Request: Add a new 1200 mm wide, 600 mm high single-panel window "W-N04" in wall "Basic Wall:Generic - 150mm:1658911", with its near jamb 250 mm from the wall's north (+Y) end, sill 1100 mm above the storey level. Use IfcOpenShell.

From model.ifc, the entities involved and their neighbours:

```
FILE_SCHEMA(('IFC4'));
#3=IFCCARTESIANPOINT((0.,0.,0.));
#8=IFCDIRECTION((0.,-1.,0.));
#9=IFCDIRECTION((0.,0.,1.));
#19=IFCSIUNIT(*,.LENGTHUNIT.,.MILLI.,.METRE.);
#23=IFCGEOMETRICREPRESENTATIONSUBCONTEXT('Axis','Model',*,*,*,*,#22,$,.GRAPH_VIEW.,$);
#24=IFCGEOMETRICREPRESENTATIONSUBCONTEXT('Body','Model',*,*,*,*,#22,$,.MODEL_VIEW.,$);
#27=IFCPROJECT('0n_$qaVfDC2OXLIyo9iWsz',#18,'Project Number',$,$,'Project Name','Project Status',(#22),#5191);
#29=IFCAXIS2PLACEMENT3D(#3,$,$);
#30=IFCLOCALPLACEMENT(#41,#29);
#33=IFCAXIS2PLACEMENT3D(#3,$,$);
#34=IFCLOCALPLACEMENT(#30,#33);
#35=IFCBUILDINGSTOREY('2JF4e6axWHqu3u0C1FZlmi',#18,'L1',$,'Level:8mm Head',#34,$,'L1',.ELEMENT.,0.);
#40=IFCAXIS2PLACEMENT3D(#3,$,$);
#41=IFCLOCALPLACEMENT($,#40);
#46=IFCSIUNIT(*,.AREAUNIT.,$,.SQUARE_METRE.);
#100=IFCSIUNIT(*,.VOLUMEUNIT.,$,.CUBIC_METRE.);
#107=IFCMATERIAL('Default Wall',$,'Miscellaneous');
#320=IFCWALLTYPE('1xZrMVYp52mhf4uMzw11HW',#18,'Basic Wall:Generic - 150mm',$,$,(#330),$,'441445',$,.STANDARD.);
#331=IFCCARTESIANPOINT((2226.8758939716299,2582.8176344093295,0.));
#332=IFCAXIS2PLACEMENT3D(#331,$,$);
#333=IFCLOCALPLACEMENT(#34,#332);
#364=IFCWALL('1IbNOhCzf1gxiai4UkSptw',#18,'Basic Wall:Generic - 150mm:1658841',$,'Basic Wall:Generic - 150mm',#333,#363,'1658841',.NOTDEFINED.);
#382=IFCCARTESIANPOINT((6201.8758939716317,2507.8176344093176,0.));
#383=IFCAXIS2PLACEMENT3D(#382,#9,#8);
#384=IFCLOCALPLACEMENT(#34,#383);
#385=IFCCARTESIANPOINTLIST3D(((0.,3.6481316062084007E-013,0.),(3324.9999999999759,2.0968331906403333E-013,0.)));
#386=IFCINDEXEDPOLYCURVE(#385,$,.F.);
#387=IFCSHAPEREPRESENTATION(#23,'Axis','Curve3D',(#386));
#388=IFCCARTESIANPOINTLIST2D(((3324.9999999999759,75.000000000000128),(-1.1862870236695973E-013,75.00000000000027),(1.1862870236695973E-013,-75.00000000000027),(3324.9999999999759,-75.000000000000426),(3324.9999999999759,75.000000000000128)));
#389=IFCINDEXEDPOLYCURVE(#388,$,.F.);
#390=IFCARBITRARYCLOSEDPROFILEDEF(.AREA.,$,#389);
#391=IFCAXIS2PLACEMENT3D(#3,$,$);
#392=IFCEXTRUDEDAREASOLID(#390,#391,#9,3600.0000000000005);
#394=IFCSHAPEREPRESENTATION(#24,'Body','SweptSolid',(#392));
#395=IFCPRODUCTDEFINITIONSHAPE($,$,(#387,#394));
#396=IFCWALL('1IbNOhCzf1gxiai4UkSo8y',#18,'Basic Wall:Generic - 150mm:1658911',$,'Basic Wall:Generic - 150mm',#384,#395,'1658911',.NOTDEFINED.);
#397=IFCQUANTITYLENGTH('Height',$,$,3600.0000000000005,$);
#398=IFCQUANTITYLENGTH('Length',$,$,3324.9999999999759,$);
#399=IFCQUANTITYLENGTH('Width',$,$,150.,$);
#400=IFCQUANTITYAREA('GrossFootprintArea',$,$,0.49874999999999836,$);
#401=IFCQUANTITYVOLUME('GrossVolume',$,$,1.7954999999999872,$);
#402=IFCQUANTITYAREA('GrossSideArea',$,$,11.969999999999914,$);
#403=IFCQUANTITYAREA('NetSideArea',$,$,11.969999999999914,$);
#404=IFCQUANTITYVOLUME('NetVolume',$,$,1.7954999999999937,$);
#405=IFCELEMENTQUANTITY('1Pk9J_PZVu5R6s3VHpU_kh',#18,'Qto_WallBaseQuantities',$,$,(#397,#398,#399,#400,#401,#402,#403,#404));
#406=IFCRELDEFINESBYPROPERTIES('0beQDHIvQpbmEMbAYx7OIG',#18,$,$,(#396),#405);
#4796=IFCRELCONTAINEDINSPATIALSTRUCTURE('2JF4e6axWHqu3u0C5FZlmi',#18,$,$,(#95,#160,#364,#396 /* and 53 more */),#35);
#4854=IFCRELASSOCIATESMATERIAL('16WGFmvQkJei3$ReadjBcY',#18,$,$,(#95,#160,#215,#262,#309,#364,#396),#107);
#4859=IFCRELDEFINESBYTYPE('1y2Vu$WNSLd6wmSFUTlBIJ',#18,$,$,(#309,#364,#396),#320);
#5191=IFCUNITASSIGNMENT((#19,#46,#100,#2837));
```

```python
import numpy as np
import ifcopenshell
import ifcopenshell.api.feature
import ifcopenshell.api.geometry
import ifcopenshell.api.pset
import ifcopenshell.api.root
import ifcopenshell.api.spatial
import ifcopenshell.geom
import ifcopenshell.util.element
import ifcopenshell.util.placement
import ifcopenshell.util.representation
import ifcopenshell.util.shape
import ifcopenshell.util.unit

model = ifcopenshell.open("model.ifc")
unit_scale = ifcopenshell.util.unit.calculate_unit_scale(model)
area_scale = ifcopenshell.util.unit.calculate_unit_scale(model, "AREAUNIT")
volume_scale = ifcopenshell.util.unit.calculate_unit_scale(model, "VOLUMEUNIT")
settings = ifcopenshell.geom.settings()


def volume(element):
    """Net volume in cubic metres, openings subtracted."""
    shape = ifcopenshell.geom.create_shape(settings, element)
    return ifcopenshell.util.shape.get_volume(shape.geometry)


wall = model.by_guid("1IbNOhCzf1gxiai4UkSo8y")
storey = ifcopenshell.util.element.get_container(wall, ifc_class="IfcBuildingStorey")
context = ifcopenshell.util.representation.get_context(model, "Model", "Body", "MODEL_VIEW")
before = volume(wall)

width, height, from_end, sill = 1.2, 0.6, 0.25, 1.1  # metres

# The wall runs along its own X axis, and the end named is its -X end.
wall_shape = ifcopenshell.geom.create_shape(settings, wall)
x, y, z = ifcopenshell.util.shape.get_vertices(wall_shape.geometry).T
start = x.min() + from_end
face, thickness = float(y.min()), float(y.max() - y.min())
wall_matrix = ifcopenshell.util.placement.get_local_placement(wall.ObjectPlacement)
level = ifcopenshell.util.placement.get_local_placement(storey.ObjectPlacement)[2, 3]


def in_wall(x, y):
    """Placement at x, y metres in the wall's axes, at sill height."""
    matrix = wall_matrix.copy()
    matrix[:, 3] = wall_matrix @ np.array([x / unit_scale, y / unit_scale, 0.0, 1.0])
    matrix[2, 3] = level + sill / unit_scale
    return matrix


# Opening: a box that overshoots both wall faces by 50 mm.
opening = ifcopenshell.api.root.create_entity(model, ifc_class="IfcOpeningElement", predefined_type="OPENING")
box = ifcopenshell.api.geometry.add_wall_representation(
    model, context=context, length=width, height=height, thickness=thickness + 0.1
)
ifcopenshell.api.geometry.assign_representation(model, product=opening, representation=box)
ifcopenshell.api.geometry.edit_object_placement(model, product=opening, matrix=in_wall(start, face - 0.05), is_si=False)
ifcopenshell.api.feature.add_feature(model, feature=opening, element=wall)

window = ifcopenshell.api.root.create_entity(model, ifc_class="IfcWindow", name="W-N04", predefined_type="WINDOW")
window.OverallWidth, window.OverallHeight = width / unit_scale, height / unit_scale
window.PartitioningType = "SINGLE_PANEL"
body = ifcopenshell.api.geometry.add_window_representation(
    model,
    context=context,
    overall_width=window.OverallWidth,
    overall_height=window.OverallHeight,
    partition_type="SINGLE_PANEL",
)
ifcopenshell.api.geometry.assign_representation(model, product=window, representation=body)
ifcopenshell.api.spatial.assign_container(model, products=[window], relating_structure=storey)
ifcopenshell.api.feature.add_filling(model, opening=opening, element=window)

# Centre the window in the wall's thickness.
ifcopenshell.api.geometry.edit_object_placement(model, product=window, matrix=in_wall(start, face), is_si=False)
window_shape = ifcopenshell.geom.create_shape(settings, window)
depth = ifcopenshell.util.shape.get_vertices(window_shape.geometry)[:, 1]
offset = face + thickness / 2 - (depth.min() + depth.max()) / 2
ifcopenshell.api.geometry.edit_object_placement(model, product=window, matrix=in_wall(start, offset), is_si=False)

after = volume(wall)

# Update the wall's stored quantities.
qto = model.by_id(ifcopenshell.util.element.get_pset(wall, "Qto_WallBaseQuantities", should_inherit=False)["id"])
ifcopenshell.api.pset.edit_qto(model, qto=qto, properties={
    "NetSideArea": after / thickness / area_scale,
    "NetVolume": after / volume_scale,
})

print(f"wall volume {before:.3f} -> {after:.3f} m3")

model.write("model_rev.ifc")
```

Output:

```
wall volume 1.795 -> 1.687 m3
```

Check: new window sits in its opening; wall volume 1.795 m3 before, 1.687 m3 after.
